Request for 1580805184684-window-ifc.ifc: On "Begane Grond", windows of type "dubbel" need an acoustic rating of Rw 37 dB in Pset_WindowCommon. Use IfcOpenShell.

First a look at what the model holds.

```python
import ifcopenshell
import ifcopenshell.util.element

model = ifcopenshell.open("1580805184684-window-ifc.ifc")
print(model.schema)
storey = next(s for s in model.by_type("IfcBuildingStorey") if s.Name == "Begane Grond")
windows = [e for e in ifcopenshell.util.element.get_decomposition(storey) if e.is_a("IfcWindow")]
seen = {}
for e in windows:
    element_type = ifcopenshell.util.element.get_type(e)
    key = (element_type.Name if element_type != e and element_type else None, ifcopenshell.util.element.get_pset(e, "Pset_WindowCommon", "AcousticRating"))
    seen[key] = seen.get(key, 0) + 1
for (name, value), count in sorted(seen.items(), key=str):
    print(count, "x", name, "|", value)
```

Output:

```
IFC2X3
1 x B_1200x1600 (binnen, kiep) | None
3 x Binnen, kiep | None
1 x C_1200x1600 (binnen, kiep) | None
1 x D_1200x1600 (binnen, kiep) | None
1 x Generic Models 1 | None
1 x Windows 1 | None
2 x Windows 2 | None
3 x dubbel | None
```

```python
import ifcopenshell
import ifcopenshell.api.pset
import ifcopenshell.util.element

model = ifcopenshell.open("1580805184684-window-ifc.ifc")

storey = next(s for s in model.by_type("IfcBuildingStorey") if s.Name == "Begane Grond")
windows = [e for e in ifcopenshell.util.element.get_decomposition(storey) if e.is_a("IfcWindow")]

count = 0
for e in windows:
    element_type = ifcopenshell.util.element.get_type(e)
    if element_type in (None, e) or element_type.Name != "dubbel":
        continue
    # add_pset returns the element's existing set when there is one.
    pset = ifcopenshell.api.pset.add_pset(model, product=e, name="Pset_WindowCommon")
    ifcopenshell.api.pset.edit_pset(model, pset=pset, properties={"AcousticRating": "Rw 37 dB"})
    count += 1

print(count, "windows updated")

model.write("1580805184684-window-ifc_updated.ifc")
```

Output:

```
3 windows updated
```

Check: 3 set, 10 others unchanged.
